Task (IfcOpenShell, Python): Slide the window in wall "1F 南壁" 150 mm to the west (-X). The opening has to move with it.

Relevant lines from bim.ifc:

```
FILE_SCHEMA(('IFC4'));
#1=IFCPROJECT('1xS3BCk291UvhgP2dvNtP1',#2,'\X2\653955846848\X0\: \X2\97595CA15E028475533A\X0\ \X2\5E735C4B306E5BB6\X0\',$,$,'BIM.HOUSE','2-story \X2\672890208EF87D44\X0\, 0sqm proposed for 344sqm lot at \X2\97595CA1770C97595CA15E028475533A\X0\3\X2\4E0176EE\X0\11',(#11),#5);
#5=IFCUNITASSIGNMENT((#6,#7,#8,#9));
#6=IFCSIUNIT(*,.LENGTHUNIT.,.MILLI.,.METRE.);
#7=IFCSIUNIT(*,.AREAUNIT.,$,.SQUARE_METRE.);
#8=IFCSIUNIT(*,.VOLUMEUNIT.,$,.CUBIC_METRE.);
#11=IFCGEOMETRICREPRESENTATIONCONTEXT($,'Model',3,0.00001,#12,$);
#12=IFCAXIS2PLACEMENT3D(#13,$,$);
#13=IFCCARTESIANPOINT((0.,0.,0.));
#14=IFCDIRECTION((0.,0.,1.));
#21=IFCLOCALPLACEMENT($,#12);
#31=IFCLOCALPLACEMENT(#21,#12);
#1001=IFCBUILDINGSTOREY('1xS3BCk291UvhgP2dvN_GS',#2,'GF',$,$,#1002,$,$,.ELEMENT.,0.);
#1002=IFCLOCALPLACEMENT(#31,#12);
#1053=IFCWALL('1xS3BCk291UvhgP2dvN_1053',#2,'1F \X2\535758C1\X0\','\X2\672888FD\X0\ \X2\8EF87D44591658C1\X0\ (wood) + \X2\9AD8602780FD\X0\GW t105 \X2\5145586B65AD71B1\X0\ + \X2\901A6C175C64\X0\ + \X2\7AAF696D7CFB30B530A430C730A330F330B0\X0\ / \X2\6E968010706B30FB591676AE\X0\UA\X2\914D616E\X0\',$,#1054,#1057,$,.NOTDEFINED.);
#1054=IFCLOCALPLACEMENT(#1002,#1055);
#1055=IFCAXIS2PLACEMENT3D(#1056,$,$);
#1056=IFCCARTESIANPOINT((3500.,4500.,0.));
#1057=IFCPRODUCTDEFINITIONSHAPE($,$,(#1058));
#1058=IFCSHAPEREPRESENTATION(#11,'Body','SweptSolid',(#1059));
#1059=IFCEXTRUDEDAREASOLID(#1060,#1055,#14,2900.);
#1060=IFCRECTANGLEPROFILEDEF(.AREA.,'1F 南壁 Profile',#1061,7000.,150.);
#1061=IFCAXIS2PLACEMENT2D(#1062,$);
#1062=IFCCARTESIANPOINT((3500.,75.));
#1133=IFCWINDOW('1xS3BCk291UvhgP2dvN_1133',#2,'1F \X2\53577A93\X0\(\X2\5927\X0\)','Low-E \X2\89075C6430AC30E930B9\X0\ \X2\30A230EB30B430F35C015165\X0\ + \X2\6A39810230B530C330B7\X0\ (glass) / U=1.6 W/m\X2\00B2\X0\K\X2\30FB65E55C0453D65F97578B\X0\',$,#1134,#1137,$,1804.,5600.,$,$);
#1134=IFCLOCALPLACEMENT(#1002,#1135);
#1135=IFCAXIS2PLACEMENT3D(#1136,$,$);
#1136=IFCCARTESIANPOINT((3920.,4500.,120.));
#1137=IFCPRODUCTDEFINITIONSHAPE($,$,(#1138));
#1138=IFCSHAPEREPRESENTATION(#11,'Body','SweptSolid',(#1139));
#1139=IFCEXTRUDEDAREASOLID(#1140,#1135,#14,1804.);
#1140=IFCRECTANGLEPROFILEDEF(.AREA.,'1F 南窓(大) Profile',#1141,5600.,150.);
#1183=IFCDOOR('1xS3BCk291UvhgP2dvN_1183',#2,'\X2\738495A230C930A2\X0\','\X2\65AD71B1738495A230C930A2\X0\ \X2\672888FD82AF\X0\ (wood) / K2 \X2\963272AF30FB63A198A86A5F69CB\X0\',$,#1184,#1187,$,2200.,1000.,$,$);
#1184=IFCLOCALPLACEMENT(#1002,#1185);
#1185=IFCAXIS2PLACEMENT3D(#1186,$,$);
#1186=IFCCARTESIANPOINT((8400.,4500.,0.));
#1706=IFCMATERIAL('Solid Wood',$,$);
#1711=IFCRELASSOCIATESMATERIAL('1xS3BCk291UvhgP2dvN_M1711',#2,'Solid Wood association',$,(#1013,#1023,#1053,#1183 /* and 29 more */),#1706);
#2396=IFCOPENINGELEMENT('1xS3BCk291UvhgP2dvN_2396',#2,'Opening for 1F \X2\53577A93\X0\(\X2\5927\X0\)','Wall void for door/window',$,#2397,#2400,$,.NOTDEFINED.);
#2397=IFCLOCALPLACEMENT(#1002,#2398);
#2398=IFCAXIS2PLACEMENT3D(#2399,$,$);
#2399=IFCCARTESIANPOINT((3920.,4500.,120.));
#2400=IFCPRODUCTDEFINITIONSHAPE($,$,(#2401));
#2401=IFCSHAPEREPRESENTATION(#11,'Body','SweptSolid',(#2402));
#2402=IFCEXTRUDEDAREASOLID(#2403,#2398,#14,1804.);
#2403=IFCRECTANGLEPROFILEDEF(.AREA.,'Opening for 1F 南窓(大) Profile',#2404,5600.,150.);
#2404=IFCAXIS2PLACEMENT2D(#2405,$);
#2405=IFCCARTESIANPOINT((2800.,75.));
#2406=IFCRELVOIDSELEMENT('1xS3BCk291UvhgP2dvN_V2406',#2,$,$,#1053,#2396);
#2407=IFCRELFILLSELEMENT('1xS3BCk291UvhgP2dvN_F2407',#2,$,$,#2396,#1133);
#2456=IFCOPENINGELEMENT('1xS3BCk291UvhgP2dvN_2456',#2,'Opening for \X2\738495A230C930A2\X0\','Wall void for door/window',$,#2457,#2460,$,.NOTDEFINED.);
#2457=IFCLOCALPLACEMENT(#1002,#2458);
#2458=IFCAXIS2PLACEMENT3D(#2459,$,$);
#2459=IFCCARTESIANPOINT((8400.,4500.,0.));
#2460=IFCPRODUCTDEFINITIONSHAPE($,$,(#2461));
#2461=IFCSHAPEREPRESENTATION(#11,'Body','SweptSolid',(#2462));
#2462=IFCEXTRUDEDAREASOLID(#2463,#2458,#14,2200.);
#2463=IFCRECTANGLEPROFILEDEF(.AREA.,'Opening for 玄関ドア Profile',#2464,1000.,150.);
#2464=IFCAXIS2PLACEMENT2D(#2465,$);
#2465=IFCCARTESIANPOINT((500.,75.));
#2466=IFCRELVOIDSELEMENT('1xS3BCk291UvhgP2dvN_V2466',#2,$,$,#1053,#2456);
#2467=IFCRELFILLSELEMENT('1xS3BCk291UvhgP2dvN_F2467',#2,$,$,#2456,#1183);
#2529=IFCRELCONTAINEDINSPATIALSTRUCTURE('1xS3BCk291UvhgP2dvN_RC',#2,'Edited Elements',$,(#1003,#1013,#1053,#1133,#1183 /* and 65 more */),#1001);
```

```python
import ifcopenshell
import ifcopenshell.api.geometry
import ifcopenshell.util.placement
import ifcopenshell.util.unit

model = ifcopenshell.open("bim.ifc")
unit_scale = ifcopenshell.util.unit.calculate_unit_scale(model)

window = model.by_guid("1xS3BCk291UvhgP2dvN_1133")
opening = window.FillsVoids[0].RelatingOpeningElement
wall = opening.VoidsElements[0].RelatingBuildingElement

wall_matrix = ifcopenshell.util.placement.get_local_placement(wall.ObjectPlacement)
shift = wall_matrix[:3, 0] * -0.15 / unit_scale
before = ifcopenshell.util.placement.get_local_placement(window.ObjectPlacement)[:3, 3].copy()

# The window is not placed relative to its opening, so move both.
for product in (opening, window):
    matrix = ifcopenshell.util.placement.get_local_placement(product.ObjectPlacement)
    matrix[:3, 3] += shift
    ifcopenshell.api.geometry.edit_object_placement(model, product=product, matrix=matrix, is_si=False)

after = ifcopenshell.util.placement.get_local_placement(window.ObjectPlacement)[:3, 3]
print("window moved by", (after - before).round(3) + 0.0)

model.write("bim_updated.ifc")
```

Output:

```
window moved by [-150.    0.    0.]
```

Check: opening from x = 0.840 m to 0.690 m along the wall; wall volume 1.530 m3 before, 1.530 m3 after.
